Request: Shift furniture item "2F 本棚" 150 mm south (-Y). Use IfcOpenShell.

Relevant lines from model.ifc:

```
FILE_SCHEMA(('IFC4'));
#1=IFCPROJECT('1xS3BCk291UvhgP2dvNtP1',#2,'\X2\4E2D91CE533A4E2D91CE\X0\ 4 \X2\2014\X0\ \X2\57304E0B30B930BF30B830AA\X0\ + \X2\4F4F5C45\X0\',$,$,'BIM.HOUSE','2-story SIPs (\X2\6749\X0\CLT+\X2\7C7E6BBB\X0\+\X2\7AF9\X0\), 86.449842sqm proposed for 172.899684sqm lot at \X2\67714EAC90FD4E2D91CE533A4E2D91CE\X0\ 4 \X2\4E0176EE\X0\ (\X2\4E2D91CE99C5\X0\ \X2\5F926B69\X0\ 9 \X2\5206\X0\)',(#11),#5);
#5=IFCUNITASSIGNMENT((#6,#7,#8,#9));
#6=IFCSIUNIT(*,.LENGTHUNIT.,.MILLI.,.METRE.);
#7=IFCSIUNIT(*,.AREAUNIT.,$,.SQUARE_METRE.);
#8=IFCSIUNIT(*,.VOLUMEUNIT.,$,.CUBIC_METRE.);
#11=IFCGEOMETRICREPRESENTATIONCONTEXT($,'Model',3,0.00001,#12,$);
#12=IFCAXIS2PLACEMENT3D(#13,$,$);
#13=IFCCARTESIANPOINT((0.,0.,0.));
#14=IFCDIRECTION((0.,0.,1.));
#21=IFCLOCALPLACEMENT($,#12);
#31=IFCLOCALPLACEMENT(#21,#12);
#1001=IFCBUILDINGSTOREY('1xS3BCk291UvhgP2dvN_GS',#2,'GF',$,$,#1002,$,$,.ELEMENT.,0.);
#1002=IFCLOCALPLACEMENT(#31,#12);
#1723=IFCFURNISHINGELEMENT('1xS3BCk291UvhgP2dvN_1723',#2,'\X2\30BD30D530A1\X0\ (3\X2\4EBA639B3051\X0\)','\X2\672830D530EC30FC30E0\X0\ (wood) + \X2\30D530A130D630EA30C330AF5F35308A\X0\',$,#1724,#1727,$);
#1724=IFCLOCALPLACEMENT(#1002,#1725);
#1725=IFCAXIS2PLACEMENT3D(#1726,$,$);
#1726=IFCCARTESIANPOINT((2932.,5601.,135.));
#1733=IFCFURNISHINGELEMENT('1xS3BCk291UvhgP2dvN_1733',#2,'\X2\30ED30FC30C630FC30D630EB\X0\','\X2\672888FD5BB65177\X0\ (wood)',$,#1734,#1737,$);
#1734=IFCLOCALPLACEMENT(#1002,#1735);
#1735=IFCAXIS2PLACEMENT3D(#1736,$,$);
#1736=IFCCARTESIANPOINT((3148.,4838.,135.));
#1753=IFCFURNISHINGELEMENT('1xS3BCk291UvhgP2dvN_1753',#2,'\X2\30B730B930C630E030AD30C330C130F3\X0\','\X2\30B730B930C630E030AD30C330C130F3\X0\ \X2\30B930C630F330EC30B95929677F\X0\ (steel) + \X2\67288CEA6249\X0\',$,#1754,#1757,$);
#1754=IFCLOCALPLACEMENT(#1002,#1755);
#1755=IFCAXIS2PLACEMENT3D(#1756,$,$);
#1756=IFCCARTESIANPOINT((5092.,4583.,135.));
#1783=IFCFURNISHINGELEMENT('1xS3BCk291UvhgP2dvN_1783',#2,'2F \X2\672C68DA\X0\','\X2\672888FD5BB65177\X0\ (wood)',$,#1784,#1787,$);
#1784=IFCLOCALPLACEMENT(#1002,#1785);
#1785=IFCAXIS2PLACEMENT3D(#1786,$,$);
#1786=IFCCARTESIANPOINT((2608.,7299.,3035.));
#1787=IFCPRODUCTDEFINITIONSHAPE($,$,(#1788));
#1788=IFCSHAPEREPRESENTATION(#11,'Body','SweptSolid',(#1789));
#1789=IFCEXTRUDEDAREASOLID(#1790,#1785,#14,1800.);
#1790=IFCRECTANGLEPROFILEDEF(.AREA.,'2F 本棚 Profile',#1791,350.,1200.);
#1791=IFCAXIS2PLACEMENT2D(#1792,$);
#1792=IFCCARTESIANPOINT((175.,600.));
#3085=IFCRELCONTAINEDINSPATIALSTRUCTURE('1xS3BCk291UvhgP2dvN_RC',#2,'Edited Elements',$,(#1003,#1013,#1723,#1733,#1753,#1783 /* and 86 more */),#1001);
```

```python
import ifcopenshell
import ifcopenshell.api.geometry
import ifcopenshell.util.placement
import ifcopenshell.util.unit

model = ifcopenshell.open("model.ifc")
unit_scale = ifcopenshell.util.unit.calculate_unit_scale(model)

item = model.by_id(1783)
matrix = ifcopenshell.util.placement.get_local_placement(item.ObjectPlacement)
matrix[1, 3] -= 0.15 / unit_scale
ifcopenshell.api.geometry.edit_object_placement(model, product=item, matrix=matrix, is_si=False)

print(ifcopenshell.util.placement.get_local_placement(item.ObjectPlacement).round(3) + 0.0)

model.write("model_updated.ifc")
```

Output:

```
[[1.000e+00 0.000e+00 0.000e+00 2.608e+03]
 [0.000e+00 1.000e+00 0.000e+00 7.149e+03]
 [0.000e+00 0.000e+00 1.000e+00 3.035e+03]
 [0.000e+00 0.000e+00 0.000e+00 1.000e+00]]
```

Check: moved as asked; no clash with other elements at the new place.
